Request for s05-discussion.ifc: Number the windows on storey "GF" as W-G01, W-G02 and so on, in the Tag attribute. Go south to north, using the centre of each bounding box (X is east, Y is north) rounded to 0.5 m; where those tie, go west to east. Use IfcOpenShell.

First a look at what the model holds.

```python
import ifcopenshell
import ifcopenshell.util.element
import ifcopenshell.util.placement

model = ifcopenshell.open("s05-discussion.ifc")
print(model.schema)
storey = next(s for s in model.by_type("IfcBuildingStorey") if s.Name == "GF")
windows = [e for e in ifcopenshell.util.element.get_decomposition(storey) if e.is_a("IfcWindow")]
for e in sorted(windows, key=lambda e: e.id()):
    origin = ifcopenshell.util.placement.get_local_placement(e.ObjectPlacement)[:3, 3]
    print(e.id(), e.Tag, e.Name, origin.round(2) + 0.0, sep=" | ")
```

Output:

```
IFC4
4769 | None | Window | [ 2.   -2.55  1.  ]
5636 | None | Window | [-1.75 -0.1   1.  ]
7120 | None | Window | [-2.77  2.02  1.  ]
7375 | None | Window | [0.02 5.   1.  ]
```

```python
import ifcopenshell
import ifcopenshell.geom
import ifcopenshell.util.element
import ifcopenshell.util.shape

model = ifcopenshell.open("s05-discussion.ifc")
settings = ifcopenshell.geom.settings()
settings.set("use-world-coords", True)


def centre(element):
    shape = ifcopenshell.geom.create_shape(settings, element)
    return ifcopenshell.util.shape.get_bbox_centroid(shape.geometry)


storey = next(s for s in model.by_type("IfcBuildingStorey") if s.Name == "GF")
windows = [e for e in ifcopenshell.util.element.get_decomposition(storey) if e.is_a("IfcWindow")]

# Insertion points can sit at a corner or the storey origin, so sort by the geometry (in metres).
centres = {e: centre(e) for e in windows}
windows.sort(key=lambda e: (round(centres[e][1] / 0.5), centres[e][0]))

for i, e in enumerate(windows, start=1):
    number = f"W-G{i:02d}"
    e.Tag = number
    print(e.id(), number)

model.write("s05-discussion_rev.ifc")
```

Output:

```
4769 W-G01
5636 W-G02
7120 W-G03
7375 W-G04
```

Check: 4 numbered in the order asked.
